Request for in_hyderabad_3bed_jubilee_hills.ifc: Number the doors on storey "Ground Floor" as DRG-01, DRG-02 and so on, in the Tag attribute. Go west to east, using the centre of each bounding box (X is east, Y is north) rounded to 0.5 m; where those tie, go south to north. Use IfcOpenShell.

First a look at what the model holds.

```python
import ifcopenshell
import ifcopenshell.util.element
import ifcopenshell.util.placement

model = ifcopenshell.open("in_hyderabad_3bed_jubilee_hills.ifc")
print(model.schema)
storey = next(s for s in model.by_type("IfcBuildingStorey") if s.Name == "Ground Floor")
doors = [e for e in ifcopenshell.util.element.get_decomposition(storey) if e.is_a("IfcDoor")]
for e in sorted(doors, key=lambda e: e.id()):
    origin = ifcopenshell.util.placement.get_local_placement(e.ObjectPlacement)[:3, 3]
    print(e.id(), e.Tag, e.Name, origin.round(2) + 0.0, sep=" | ")
```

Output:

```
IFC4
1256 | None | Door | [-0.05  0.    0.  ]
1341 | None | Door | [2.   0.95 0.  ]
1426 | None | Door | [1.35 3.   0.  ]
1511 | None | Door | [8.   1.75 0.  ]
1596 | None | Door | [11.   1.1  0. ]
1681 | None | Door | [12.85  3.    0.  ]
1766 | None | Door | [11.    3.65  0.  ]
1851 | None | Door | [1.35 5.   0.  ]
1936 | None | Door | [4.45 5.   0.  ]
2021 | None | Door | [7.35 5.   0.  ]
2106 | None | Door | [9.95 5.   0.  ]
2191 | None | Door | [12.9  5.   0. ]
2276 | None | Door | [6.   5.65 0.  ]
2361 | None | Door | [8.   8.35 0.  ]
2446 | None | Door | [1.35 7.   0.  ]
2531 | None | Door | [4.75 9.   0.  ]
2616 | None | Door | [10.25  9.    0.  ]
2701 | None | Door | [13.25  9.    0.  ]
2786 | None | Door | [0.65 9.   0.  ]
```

```python
import ifcopenshell
import ifcopenshell.geom
import ifcopenshell.util.element
import ifcopenshell.util.shape

model = ifcopenshell.open("in_hyderabad_3bed_jubilee_hills.ifc")
settings = ifcopenshell.geom.settings()
settings.set("use-world-coords", True)


def centre(element):
    shape = ifcopenshell.geom.create_shape(settings, element)
    return ifcopenshell.util.shape.get_bbox_centroid(shape.geometry)


storey = next(s for s in model.by_type("IfcBuildingStorey") if s.Name == "Ground Floor")
doors = [e for e in ifcopenshell.util.element.get_decomposition(storey) if e.is_a("IfcDoor")]

# Insertion points can sit at a corner or the storey origin, so sort by the geometry (in metres).
centres = {e: centre(e) for e in doors}
doors.sort(key=lambda e: (round(centres[e][0] / 0.5), centres[e][1]))

for i, e in enumerate(doors, start=1):
    number = f"DRG-{i:02d}"
    e.Tag = number
    print(e.id(), number)

model.write("in_hyderabad_3bed_jubilee_hills_updated.ifc")
```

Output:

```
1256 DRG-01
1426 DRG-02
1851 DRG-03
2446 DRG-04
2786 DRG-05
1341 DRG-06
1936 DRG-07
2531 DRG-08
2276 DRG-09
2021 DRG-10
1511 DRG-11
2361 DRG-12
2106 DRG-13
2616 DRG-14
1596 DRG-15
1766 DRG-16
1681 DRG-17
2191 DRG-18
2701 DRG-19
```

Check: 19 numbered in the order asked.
